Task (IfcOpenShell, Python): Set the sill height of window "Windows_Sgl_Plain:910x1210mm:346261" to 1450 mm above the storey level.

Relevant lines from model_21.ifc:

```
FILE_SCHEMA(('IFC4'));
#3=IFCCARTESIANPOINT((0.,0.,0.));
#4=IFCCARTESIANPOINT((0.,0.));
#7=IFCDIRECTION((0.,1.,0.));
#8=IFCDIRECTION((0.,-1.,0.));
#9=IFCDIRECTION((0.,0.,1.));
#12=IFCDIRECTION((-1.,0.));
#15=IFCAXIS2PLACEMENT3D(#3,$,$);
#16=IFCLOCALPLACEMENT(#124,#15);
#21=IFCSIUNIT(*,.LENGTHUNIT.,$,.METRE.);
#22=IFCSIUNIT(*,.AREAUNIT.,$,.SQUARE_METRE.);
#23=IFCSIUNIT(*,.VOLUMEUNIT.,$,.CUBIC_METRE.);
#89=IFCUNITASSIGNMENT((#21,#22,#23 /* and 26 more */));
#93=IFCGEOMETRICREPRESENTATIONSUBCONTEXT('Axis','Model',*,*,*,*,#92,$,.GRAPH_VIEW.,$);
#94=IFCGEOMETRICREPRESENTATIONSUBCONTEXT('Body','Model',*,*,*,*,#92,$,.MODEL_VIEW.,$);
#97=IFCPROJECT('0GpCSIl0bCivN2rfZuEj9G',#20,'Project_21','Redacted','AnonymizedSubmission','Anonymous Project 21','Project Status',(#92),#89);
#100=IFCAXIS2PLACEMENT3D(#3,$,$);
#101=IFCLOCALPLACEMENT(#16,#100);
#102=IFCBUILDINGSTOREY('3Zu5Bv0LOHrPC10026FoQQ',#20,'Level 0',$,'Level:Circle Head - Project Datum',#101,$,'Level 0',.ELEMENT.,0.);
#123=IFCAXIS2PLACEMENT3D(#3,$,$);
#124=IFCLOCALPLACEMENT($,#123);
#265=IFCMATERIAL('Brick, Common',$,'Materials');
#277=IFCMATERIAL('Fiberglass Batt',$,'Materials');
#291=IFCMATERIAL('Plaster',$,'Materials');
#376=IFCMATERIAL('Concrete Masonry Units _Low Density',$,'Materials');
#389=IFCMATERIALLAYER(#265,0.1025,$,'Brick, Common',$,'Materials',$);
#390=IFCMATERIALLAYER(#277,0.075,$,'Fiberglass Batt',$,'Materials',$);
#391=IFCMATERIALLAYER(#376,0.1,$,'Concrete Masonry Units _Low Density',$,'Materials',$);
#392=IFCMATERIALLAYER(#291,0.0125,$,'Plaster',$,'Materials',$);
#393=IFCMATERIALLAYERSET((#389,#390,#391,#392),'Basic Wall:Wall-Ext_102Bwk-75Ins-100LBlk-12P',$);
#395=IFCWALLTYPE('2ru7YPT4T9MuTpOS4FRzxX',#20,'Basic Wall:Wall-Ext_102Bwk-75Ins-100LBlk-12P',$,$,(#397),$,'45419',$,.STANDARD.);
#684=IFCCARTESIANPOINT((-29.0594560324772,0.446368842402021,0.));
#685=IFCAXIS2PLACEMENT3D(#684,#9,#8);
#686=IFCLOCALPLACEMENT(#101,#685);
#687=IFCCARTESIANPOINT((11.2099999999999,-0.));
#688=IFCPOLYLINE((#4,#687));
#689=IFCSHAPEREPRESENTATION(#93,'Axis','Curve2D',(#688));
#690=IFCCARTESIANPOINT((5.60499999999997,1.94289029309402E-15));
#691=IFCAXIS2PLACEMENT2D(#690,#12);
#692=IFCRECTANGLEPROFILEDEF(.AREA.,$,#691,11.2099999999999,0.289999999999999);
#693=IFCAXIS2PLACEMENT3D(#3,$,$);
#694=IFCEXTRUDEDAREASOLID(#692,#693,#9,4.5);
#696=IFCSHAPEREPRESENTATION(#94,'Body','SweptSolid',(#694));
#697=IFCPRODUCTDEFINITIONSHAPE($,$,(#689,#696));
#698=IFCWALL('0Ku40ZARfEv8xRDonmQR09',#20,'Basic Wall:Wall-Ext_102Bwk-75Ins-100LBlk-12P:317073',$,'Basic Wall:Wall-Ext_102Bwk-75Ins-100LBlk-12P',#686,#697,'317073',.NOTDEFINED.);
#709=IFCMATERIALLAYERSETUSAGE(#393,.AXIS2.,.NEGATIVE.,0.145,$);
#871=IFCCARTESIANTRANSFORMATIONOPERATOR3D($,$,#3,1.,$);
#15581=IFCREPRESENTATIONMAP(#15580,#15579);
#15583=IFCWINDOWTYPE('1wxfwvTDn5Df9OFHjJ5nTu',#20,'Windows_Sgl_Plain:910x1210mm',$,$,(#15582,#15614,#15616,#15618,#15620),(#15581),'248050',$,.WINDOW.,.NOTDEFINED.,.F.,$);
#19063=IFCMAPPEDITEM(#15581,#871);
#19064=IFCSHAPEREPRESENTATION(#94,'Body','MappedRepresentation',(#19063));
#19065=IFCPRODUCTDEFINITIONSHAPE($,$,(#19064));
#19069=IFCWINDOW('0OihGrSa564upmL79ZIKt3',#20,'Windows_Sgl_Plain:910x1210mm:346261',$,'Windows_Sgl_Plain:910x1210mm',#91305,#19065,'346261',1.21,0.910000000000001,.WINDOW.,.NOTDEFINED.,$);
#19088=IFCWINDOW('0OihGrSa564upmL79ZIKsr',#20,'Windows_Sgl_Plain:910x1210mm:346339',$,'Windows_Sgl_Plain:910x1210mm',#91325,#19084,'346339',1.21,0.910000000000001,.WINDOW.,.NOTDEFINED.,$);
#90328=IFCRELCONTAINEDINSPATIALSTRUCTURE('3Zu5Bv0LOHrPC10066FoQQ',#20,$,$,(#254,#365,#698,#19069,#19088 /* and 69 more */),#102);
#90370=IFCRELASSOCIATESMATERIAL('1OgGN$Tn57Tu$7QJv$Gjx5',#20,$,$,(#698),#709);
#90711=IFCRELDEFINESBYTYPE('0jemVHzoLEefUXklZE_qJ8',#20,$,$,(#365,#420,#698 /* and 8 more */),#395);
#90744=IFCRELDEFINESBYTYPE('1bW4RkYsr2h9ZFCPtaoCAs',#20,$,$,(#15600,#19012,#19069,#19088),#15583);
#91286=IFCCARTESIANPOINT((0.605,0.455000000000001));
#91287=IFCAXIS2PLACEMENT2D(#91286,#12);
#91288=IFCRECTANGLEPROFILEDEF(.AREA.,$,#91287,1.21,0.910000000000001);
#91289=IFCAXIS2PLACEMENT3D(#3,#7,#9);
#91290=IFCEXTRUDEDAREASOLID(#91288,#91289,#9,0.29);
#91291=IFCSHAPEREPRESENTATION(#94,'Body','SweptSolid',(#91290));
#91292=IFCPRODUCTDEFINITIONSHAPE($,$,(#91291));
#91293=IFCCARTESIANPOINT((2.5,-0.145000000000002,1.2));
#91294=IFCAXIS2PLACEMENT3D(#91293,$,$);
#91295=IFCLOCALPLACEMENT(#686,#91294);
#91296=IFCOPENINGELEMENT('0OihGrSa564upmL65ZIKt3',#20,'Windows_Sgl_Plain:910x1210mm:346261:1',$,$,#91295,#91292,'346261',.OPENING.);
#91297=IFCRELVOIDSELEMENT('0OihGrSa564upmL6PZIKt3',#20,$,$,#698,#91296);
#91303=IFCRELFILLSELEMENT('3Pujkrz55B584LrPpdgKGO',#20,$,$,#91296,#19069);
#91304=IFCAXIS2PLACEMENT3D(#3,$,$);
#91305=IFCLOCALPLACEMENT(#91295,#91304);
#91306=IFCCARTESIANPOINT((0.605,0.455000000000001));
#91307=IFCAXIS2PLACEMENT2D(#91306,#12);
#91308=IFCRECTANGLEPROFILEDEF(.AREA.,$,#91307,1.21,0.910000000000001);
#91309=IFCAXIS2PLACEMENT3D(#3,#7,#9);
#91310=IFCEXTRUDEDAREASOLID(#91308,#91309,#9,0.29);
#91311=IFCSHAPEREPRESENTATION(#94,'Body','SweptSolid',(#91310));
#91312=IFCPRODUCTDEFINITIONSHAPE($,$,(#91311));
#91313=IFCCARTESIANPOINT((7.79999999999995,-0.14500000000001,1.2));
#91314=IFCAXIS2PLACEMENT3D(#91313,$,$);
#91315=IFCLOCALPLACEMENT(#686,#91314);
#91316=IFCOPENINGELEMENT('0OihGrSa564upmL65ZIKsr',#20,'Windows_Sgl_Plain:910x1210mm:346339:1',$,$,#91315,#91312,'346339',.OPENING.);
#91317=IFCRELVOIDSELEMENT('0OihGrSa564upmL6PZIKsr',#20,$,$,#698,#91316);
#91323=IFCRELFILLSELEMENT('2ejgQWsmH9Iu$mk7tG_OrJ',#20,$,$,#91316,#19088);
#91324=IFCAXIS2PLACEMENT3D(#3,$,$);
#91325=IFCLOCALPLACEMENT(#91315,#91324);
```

```python
import numpy as np
import ifcopenshell
import ifcopenshell.api.geometry
import ifcopenshell.geom
import ifcopenshell.util.element
import ifcopenshell.util.placement
import ifcopenshell.util.shape
import ifcopenshell.util.unit

model = ifcopenshell.open("model_21.ifc")
unit_scale = ifcopenshell.util.unit.calculate_unit_scale(model)

window = model.by_guid("0OihGrSa564upmL79ZIKt3")
opening = window.FillsVoids[0].RelatingOpeningElement
storey = ifcopenshell.util.element.get_container(window, ifc_class="IfcBuildingStorey")
level = ifcopenshell.util.placement.get_local_placement(storey.ObjectPlacement)[2, 3]

# The opening's origin need not be at the sill, so measure its lowest point.
shape = ifcopenshell.geom.create_shape(ifcopenshell.geom.settings(), opening)
bottom = ifcopenshell.util.shape.get_shape_bottom_elevation(shape, shape.geometry) / unit_scale
dz = level + 1.45 - bottom

shift = np.array([0.0, 0.0, dz])
# The window is placed relative to its opening, so it follows when the opening moves.
matrix = ifcopenshell.util.placement.get_local_placement(opening.ObjectPlacement)
matrix[:3, 3] += shift
ifcopenshell.api.geometry.edit_object_placement(
    model, product=opening, matrix=matrix, is_si=False, should_transform_children=True
)

print(f"moved by {dz * unit_scale:+.3f} m")

model.write("model_21_rev.ifc")
```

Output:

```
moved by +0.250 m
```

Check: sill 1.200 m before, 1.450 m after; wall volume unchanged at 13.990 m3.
